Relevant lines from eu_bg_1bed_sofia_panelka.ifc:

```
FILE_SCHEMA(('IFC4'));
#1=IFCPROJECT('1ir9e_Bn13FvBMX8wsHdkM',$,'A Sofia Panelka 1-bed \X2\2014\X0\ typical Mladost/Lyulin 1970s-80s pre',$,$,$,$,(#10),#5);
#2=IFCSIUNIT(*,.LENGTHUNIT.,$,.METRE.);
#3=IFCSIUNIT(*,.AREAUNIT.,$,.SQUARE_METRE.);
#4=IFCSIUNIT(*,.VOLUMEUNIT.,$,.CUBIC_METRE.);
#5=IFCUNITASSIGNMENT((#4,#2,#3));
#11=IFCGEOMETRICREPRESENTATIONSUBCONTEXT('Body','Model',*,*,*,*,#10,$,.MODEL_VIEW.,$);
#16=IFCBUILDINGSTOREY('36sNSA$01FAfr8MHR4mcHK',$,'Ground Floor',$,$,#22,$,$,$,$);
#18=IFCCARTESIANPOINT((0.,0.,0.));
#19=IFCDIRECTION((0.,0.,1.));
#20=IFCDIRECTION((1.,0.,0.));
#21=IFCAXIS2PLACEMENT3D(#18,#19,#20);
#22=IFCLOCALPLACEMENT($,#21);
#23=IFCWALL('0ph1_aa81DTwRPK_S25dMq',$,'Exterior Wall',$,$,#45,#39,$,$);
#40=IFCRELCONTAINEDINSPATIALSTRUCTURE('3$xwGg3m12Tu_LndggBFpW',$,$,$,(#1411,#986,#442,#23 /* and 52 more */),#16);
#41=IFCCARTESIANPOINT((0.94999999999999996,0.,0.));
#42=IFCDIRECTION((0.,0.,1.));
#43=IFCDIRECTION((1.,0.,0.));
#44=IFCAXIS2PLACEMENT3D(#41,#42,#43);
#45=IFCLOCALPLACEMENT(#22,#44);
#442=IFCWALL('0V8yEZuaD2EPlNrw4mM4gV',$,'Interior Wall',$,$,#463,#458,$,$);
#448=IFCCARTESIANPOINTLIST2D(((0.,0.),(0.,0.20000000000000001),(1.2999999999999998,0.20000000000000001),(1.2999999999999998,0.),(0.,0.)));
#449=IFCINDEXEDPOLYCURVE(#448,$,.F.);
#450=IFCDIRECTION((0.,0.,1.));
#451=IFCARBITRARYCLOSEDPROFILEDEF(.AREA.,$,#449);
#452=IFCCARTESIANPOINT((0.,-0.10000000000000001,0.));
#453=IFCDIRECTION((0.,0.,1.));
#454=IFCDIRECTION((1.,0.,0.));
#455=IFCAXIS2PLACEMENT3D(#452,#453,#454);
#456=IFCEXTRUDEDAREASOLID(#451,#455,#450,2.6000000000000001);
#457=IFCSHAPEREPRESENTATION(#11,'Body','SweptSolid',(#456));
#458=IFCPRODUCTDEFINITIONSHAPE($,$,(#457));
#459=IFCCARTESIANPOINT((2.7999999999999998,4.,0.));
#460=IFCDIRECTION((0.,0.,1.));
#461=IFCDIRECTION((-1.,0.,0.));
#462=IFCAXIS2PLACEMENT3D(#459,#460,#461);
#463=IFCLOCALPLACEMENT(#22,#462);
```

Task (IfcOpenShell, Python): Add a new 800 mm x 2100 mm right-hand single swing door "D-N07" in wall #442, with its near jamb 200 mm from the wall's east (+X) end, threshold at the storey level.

```python
import numpy as np
import ifcopenshell
import ifcopenshell.api.feature
import ifcopenshell.api.geometry
import ifcopenshell.api.root
import ifcopenshell.api.spatial
import ifcopenshell.geom
import ifcopenshell.util.element
import ifcopenshell.util.placement
import ifcopenshell.util.representation
import ifcopenshell.util.shape
import ifcopenshell.util.unit

model = ifcopenshell.open("eu_bg_1bed_sofia_panelka.ifc")
unit_scale = ifcopenshell.util.unit.calculate_unit_scale(model)
settings = ifcopenshell.geom.settings()


def volume(element):
    """Net volume in cubic metres, openings subtracted."""
    shape = ifcopenshell.geom.create_shape(settings, element)
    return ifcopenshell.util.shape.get_volume(shape.geometry)


wall = model.by_id(442)
storey = ifcopenshell.util.element.get_container(wall, ifc_class="IfcBuildingStorey")
context = ifcopenshell.util.representation.get_context(model, "Model", "Body", "MODEL_VIEW")
before = volume(wall)

width, height, from_end, sill = 0.8, 2.1, 0.2, 0.0  # metres

# The wall runs along its own X axis, and the end named is its -X end.
wall_shape = ifcopenshell.geom.create_shape(settings, wall)
x, y, z = ifcopenshell.util.shape.get_vertices(wall_shape.geometry).T
start = x.min() + from_end
face, thickness = float(y.min()), float(y.max() - y.min())
wall_matrix = ifcopenshell.util.placement.get_local_placement(wall.ObjectPlacement)
level = ifcopenshell.util.placement.get_local_placement(storey.ObjectPlacement)[2, 3]


def in_wall(x, y):
    """Placement at x, y metres in the wall's axes, at sill height."""
    matrix = wall_matrix.copy()
    matrix[:, 3] = wall_matrix @ np.array([x / unit_scale, y / unit_scale, 0.0, 1.0])
    matrix[2, 3] = level + sill / unit_scale
    return matrix


# Opening: a box that overshoots both wall faces by 50 mm.
opening = ifcopenshell.api.root.create_entity(model, ifc_class="IfcOpeningElement", predefined_type="OPENING")
box = ifcopenshell.api.geometry.add_wall_representation(
    model, context=context, length=width, height=height, thickness=thickness + 0.1
)
ifcopenshell.api.geometry.assign_representation(model, product=opening, representation=box)
ifcopenshell.api.geometry.edit_object_placement(model, product=opening, matrix=in_wall(start, face - 0.05), is_si=False)
ifcopenshell.api.feature.add_feature(model, feature=opening, element=wall)

door = ifcopenshell.api.root.create_entity(model, ifc_class="IfcDoor", name="D-N07", predefined_type="DOOR")
door.OverallWidth, door.OverallHeight = width / unit_scale, height / unit_scale
door.OperationType = "SINGLE_SWING_RIGHT"
body = ifcopenshell.api.geometry.add_door_representation(
    model,
    context=context,
    overall_width=door.OverallWidth,
    overall_height=door.OverallHeight,
    operation_type="SINGLE_SWING_RIGHT",
    lining_properties={"LiningDepth": thickness / unit_scale, "ThresholdDepth": thickness / unit_scale},
)
ifcopenshell.api.geometry.assign_representation(model, product=door, representation=body)
ifcopenshell.api.spatial.assign_container(model, products=[door], relating_structure=storey)
ifcopenshell.api.feature.add_filling(model, opening=opening, element=door)

# The lining spans the wall, so the door starts at the wall face.
ifcopenshell.api.geometry.edit_object_placement(model, product=door, matrix=in_wall(start, face), is_si=False)

after = volume(wall)

print(f"wall volume {before:.3f} -> {after:.3f} m3")

model.write("eu_bg_1bed_sofia_panelka_rev.ifc")
```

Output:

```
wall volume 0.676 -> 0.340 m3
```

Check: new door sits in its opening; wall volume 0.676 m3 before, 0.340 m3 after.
